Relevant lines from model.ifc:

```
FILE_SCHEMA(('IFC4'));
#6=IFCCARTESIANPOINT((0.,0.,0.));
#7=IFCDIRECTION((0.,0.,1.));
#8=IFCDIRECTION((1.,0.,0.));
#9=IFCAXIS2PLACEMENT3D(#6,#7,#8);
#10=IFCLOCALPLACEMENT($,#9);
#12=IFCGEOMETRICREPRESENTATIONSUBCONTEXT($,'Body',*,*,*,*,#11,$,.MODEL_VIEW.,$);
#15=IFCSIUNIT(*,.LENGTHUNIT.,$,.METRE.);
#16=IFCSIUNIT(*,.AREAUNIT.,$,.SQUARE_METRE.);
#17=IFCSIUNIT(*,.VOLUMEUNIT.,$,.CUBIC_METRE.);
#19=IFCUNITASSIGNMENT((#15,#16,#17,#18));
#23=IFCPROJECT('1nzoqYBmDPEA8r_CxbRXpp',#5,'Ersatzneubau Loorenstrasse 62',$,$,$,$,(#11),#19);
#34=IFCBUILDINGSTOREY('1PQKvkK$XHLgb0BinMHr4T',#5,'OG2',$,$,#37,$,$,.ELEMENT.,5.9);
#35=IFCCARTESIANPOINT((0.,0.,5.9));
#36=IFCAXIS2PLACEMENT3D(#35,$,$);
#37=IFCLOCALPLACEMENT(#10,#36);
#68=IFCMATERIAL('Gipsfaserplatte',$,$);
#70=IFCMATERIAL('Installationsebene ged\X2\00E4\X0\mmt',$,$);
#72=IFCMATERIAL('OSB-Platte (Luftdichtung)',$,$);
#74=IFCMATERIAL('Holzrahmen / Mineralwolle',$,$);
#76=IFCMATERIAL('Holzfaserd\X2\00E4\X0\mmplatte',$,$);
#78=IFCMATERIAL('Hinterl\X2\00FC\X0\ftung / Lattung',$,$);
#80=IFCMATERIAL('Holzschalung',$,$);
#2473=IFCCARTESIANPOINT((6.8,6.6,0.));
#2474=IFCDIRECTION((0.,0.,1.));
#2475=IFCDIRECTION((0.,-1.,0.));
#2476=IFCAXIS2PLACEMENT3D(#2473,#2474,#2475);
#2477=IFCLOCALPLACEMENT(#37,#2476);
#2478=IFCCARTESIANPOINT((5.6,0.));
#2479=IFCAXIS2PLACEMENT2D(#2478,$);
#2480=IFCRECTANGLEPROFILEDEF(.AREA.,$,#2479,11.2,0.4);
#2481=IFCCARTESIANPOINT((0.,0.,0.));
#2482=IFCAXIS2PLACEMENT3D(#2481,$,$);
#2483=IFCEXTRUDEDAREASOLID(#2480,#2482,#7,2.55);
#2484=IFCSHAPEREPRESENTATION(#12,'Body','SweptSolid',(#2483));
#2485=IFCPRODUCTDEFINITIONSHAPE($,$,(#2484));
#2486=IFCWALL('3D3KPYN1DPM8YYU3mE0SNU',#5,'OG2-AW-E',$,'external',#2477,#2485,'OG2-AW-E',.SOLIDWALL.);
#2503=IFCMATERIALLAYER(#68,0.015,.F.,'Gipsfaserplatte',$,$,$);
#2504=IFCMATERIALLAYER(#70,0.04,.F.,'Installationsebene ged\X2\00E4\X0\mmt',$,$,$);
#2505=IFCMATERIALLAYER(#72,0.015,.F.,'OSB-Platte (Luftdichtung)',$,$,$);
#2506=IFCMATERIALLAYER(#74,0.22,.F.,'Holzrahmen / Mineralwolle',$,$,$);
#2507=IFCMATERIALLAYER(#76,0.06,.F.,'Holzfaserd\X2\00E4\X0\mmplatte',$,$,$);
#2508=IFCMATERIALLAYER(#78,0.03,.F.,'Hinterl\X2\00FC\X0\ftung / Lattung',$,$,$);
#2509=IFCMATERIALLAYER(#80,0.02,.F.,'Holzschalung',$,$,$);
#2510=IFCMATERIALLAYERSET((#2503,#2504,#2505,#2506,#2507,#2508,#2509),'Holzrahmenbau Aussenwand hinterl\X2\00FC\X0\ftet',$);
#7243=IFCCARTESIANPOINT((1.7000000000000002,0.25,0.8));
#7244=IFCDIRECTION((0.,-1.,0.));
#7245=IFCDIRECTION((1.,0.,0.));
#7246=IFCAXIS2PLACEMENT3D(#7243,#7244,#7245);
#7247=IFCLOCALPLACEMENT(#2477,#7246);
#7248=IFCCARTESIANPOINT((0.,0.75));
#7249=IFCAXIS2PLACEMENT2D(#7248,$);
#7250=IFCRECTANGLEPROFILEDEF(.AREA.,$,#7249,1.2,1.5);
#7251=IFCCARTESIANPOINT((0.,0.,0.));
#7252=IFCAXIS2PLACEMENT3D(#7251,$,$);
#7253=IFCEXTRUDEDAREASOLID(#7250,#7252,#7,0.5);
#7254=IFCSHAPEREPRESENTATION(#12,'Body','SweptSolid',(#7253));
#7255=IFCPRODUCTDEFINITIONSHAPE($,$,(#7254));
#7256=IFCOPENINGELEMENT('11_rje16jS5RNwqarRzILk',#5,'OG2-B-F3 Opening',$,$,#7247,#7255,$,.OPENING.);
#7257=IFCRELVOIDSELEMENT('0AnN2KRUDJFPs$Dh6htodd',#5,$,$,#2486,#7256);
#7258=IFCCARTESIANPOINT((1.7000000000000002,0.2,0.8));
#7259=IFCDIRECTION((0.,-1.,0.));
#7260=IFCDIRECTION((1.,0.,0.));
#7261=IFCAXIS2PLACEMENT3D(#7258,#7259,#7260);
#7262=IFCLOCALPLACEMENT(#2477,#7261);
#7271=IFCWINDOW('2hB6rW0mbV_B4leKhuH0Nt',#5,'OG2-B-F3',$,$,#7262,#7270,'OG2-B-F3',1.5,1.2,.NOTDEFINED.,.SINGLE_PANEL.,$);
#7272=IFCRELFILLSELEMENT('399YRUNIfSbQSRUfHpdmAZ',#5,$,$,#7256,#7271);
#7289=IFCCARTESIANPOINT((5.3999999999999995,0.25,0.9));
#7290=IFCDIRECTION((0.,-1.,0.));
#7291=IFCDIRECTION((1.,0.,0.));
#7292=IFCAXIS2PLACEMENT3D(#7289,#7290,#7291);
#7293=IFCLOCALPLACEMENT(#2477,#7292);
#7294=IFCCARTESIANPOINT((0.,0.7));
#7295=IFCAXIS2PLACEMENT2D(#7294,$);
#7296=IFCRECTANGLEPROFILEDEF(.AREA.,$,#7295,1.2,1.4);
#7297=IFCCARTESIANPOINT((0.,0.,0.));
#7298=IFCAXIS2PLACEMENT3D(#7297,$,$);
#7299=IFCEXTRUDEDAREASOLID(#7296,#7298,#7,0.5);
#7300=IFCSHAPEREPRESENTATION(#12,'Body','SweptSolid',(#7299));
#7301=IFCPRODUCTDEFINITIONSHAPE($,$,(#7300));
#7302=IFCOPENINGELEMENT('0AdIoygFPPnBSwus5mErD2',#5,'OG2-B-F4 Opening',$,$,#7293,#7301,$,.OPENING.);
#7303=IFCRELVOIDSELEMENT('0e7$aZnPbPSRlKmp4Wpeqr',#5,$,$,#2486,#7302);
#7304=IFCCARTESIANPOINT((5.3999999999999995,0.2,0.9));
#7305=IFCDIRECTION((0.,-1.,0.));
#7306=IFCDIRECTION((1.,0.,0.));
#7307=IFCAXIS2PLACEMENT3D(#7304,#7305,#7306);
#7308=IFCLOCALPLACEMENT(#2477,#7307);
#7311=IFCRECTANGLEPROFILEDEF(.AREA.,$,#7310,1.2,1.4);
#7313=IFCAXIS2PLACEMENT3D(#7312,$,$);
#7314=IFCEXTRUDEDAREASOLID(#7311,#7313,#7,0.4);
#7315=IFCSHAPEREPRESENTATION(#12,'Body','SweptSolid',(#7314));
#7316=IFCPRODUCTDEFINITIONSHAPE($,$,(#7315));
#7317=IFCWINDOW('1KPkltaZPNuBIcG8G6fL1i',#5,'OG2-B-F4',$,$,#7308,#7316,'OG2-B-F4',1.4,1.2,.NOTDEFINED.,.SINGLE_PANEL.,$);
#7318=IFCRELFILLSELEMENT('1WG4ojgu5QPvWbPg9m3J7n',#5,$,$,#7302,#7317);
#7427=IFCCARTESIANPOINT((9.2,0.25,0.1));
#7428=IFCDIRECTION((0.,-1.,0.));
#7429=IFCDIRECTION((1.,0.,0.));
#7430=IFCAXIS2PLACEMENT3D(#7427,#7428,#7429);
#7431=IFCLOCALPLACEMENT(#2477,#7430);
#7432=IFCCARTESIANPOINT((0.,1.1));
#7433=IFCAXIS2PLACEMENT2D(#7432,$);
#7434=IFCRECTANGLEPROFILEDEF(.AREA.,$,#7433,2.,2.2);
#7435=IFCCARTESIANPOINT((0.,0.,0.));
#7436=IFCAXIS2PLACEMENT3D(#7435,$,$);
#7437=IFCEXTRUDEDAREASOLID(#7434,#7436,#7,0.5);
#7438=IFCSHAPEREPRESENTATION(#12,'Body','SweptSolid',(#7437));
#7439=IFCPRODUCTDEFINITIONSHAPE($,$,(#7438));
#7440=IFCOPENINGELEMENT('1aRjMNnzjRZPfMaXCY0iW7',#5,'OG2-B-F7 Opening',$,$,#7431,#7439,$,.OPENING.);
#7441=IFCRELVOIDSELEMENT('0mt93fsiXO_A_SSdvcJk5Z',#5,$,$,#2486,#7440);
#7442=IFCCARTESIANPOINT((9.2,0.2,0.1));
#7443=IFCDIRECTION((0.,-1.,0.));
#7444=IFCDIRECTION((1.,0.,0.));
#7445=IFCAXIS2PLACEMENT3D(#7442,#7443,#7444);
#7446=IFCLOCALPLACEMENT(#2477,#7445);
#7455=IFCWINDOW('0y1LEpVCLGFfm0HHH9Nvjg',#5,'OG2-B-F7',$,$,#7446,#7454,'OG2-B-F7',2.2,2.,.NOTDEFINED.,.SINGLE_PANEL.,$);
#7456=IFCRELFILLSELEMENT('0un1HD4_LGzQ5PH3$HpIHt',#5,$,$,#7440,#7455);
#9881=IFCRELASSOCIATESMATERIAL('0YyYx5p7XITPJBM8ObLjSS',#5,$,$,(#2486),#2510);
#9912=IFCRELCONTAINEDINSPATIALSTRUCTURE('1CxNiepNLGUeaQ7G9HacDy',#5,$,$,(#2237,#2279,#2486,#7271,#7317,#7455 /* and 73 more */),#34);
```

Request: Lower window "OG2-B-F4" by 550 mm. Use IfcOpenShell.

```python
import numpy as np
import ifcopenshell
import ifcopenshell.api.geometry
import ifcopenshell.util.placement
import ifcopenshell.util.unit

model = ifcopenshell.open("model.ifc")
unit_scale = ifcopenshell.util.unit.calculate_unit_scale(model)

window = model.by_id(7317)
opening = window.FillsVoids[0].RelatingOpeningElement
dz = -0.55 / unit_scale

shift = np.array([0.0, 0.0, dz])
# The window is not placed relative to its opening, so move both.
for product in (opening, window):
    matrix = ifcopenshell.util.placement.get_local_placement(product.ObjectPlacement)
    matrix[:3, 3] += shift
    ifcopenshell.api.geometry.edit_object_placement(model, product=product, matrix=matrix, is_si=False)

print(f"moved by {dz * unit_scale:+.3f} m")

model.write("model_v2.ifc")
```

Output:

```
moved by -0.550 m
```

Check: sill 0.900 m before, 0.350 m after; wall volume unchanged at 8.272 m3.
